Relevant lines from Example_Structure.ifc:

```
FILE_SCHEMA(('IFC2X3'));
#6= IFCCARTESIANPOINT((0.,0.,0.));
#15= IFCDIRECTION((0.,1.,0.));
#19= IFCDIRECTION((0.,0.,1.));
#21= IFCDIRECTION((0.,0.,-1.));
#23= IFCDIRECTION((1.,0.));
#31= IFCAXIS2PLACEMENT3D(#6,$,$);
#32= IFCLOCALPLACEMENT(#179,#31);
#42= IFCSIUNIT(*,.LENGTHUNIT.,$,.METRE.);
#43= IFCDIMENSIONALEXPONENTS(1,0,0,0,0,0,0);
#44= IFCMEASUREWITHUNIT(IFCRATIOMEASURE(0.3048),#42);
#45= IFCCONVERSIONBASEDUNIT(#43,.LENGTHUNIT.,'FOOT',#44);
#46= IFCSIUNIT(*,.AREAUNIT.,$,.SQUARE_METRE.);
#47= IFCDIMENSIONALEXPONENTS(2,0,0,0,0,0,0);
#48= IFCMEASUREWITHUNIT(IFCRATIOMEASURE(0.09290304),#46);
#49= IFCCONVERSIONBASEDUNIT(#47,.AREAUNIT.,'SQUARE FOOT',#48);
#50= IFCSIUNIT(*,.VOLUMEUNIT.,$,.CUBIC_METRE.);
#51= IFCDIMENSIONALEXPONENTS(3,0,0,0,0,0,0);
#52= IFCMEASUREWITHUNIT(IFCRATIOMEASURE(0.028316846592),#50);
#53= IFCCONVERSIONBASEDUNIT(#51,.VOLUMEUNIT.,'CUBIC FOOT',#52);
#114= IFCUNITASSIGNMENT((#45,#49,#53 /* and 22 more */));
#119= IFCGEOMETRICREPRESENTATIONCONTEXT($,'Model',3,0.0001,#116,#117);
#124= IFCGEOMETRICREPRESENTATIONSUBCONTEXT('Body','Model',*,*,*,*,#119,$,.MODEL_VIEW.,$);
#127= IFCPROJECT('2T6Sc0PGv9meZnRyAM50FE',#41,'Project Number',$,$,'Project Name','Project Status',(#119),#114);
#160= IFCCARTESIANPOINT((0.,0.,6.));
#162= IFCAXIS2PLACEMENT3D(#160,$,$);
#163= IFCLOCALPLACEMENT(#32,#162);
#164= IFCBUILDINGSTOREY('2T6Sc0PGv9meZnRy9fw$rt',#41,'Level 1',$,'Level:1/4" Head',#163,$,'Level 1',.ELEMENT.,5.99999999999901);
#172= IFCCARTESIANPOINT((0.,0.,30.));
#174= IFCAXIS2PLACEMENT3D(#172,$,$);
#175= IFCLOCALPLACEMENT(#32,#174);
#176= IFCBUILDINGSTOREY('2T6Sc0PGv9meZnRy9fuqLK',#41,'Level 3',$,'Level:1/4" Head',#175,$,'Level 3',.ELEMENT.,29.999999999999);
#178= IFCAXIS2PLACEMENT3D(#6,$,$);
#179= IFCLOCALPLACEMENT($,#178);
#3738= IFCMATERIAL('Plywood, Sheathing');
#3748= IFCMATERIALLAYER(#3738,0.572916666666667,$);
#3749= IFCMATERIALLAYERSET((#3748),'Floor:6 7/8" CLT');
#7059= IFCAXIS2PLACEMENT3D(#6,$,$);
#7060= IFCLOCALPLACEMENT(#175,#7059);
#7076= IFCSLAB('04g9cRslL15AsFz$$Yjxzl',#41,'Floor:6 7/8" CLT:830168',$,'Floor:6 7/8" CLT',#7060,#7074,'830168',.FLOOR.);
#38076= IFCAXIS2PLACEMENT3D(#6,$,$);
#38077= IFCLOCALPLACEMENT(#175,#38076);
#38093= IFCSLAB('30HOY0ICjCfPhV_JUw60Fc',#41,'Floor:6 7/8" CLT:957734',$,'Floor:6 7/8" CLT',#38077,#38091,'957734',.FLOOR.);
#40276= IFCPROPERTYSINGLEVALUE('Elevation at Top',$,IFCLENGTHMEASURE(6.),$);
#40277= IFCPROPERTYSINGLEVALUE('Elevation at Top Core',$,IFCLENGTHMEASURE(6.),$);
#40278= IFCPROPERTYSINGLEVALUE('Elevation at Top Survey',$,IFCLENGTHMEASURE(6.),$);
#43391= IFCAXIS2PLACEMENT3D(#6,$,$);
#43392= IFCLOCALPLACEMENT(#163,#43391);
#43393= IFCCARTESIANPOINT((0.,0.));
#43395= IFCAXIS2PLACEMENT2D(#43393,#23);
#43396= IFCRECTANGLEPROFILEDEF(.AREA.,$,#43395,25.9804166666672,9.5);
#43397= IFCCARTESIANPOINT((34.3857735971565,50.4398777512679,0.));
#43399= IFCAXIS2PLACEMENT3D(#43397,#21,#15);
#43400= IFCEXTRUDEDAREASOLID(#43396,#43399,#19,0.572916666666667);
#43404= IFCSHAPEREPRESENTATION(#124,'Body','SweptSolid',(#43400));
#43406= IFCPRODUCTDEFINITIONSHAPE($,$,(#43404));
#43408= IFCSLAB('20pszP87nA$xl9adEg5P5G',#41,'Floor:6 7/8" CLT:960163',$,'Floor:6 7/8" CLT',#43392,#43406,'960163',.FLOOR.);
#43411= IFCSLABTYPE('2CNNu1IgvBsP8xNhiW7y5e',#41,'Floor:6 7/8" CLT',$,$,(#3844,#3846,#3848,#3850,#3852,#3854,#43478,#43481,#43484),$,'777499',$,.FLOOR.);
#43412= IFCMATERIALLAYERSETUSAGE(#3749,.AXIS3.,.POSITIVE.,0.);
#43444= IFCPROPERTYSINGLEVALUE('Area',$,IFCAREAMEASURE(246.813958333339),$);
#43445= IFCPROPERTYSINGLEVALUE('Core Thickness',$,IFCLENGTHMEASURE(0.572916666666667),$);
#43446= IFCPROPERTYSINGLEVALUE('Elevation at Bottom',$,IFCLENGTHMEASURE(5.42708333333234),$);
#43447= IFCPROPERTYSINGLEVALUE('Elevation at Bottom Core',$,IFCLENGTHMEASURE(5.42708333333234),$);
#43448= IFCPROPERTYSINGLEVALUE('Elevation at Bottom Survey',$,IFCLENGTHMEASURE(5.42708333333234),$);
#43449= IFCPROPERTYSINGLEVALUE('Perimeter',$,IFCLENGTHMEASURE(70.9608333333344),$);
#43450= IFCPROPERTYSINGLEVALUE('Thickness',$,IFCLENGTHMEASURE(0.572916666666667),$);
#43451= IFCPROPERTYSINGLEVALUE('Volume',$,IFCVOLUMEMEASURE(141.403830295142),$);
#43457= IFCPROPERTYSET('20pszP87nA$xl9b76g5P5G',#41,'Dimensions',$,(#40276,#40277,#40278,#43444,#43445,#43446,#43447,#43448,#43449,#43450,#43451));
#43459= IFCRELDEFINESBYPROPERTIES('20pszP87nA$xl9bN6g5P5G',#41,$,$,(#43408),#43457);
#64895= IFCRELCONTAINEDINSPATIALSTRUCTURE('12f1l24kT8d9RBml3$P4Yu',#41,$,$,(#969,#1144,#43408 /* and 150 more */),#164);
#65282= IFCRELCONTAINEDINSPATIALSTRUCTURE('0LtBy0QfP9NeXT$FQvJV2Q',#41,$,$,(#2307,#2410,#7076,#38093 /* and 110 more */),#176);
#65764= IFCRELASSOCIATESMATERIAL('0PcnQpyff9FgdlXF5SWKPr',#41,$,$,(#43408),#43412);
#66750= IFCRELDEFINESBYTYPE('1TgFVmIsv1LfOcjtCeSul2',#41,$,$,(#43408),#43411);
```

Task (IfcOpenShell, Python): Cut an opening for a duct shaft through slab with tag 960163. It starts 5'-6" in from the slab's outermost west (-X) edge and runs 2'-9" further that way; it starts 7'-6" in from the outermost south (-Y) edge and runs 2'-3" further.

```python
import numpy as np
import ifcopenshell
import ifcopenshell.api.feature
import ifcopenshell.api.geometry
import ifcopenshell.api.pset
import ifcopenshell.api.root
import ifcopenshell.geom
import ifcopenshell.util.element
import ifcopenshell.util.placement
import ifcopenshell.util.representation
import ifcopenshell.util.shape
import ifcopenshell.util.unit

model = ifcopenshell.open("Example_Structure.ifc")
unit_scale = ifcopenshell.util.unit.calculate_unit_scale(model)
area_scale = ifcopenshell.util.unit.calculate_unit_scale(model, "AREAUNIT")
volume_scale = ifcopenshell.util.unit.calculate_unit_scale(model, "VOLUMEUNIT")
settings = ifcopenshell.geom.settings()


def volume(element):
    """Net volume in cubic metres, openings subtracted."""
    shape = ifcopenshell.geom.create_shape(settings, element)
    return ifcopenshell.util.shape.get_volume(shape.geometry)


slab = model.by_id(43408)
before = volume(slab)

# Extent in the slab's own axes, in metres. The edges named are its -X and -Y sides.
slab_shape = ifcopenshell.geom.create_shape(settings, slab)
vertices = ifcopenshell.util.shape.get_vertices(slab_shape.geometry)
x_min, y_min, bottom = vertices.min(axis=0)
top = vertices[:, 2].max()

opening = ifcopenshell.api.root.create_entity(model, ifc_class="IfcOpeningElement", name="Duct shaft opening")
context = ifcopenshell.util.representation.get_context(model, "Model", "Body", "MODEL_VIEW")
width, depth = 0.8382, 0.6858
outline = [(0.0, 0.0), (width, 0.0), (width, depth), (0.0, depth), (0.0, 0.0)]
# Overshoot both faces by 50 mm so the cut is clean.
shape = ifcopenshell.api.geometry.add_slab_representation(
    model, context=context, depth=top - bottom + 0.1, polyline=outline
)
ifcopenshell.api.geometry.assign_representation(model, product=opening, representation=shape)

matrix = ifcopenshell.util.placement.get_local_placement(slab.ObjectPlacement)
matrix[:, 3] = matrix @ np.append(np.array([x_min + 1.6764, y_min + 2.286, bottom - 0.05]) / unit_scale, 1.0)
ifcopenshell.api.geometry.edit_object_placement(model, product=opening, matrix=matrix, is_si=False)
ifcopenshell.api.feature.add_feature(model, feature=opening, element=slab)

after = volume(slab)

# Update the slab's stored quantities.
pset = model.by_id(ifcopenshell.util.element.get_pset(slab, "Dimensions", should_inherit=False)["id"])
ifcopenshell.api.pset.edit_pset(model, pset=pset, properties={
    "Area": model.create_entity("IfcAreaMeasure", after / (top - bottom) / area_scale),
    "Volume": model.create_entity("IfcVolumeMeasure", after / volume_scale),
})

print(f"slab volume {before:.3f} -> {after:.3f} m3")

model.write("Example_Structure_rev.ifc")
```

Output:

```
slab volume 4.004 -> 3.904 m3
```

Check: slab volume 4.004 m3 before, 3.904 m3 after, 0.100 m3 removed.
